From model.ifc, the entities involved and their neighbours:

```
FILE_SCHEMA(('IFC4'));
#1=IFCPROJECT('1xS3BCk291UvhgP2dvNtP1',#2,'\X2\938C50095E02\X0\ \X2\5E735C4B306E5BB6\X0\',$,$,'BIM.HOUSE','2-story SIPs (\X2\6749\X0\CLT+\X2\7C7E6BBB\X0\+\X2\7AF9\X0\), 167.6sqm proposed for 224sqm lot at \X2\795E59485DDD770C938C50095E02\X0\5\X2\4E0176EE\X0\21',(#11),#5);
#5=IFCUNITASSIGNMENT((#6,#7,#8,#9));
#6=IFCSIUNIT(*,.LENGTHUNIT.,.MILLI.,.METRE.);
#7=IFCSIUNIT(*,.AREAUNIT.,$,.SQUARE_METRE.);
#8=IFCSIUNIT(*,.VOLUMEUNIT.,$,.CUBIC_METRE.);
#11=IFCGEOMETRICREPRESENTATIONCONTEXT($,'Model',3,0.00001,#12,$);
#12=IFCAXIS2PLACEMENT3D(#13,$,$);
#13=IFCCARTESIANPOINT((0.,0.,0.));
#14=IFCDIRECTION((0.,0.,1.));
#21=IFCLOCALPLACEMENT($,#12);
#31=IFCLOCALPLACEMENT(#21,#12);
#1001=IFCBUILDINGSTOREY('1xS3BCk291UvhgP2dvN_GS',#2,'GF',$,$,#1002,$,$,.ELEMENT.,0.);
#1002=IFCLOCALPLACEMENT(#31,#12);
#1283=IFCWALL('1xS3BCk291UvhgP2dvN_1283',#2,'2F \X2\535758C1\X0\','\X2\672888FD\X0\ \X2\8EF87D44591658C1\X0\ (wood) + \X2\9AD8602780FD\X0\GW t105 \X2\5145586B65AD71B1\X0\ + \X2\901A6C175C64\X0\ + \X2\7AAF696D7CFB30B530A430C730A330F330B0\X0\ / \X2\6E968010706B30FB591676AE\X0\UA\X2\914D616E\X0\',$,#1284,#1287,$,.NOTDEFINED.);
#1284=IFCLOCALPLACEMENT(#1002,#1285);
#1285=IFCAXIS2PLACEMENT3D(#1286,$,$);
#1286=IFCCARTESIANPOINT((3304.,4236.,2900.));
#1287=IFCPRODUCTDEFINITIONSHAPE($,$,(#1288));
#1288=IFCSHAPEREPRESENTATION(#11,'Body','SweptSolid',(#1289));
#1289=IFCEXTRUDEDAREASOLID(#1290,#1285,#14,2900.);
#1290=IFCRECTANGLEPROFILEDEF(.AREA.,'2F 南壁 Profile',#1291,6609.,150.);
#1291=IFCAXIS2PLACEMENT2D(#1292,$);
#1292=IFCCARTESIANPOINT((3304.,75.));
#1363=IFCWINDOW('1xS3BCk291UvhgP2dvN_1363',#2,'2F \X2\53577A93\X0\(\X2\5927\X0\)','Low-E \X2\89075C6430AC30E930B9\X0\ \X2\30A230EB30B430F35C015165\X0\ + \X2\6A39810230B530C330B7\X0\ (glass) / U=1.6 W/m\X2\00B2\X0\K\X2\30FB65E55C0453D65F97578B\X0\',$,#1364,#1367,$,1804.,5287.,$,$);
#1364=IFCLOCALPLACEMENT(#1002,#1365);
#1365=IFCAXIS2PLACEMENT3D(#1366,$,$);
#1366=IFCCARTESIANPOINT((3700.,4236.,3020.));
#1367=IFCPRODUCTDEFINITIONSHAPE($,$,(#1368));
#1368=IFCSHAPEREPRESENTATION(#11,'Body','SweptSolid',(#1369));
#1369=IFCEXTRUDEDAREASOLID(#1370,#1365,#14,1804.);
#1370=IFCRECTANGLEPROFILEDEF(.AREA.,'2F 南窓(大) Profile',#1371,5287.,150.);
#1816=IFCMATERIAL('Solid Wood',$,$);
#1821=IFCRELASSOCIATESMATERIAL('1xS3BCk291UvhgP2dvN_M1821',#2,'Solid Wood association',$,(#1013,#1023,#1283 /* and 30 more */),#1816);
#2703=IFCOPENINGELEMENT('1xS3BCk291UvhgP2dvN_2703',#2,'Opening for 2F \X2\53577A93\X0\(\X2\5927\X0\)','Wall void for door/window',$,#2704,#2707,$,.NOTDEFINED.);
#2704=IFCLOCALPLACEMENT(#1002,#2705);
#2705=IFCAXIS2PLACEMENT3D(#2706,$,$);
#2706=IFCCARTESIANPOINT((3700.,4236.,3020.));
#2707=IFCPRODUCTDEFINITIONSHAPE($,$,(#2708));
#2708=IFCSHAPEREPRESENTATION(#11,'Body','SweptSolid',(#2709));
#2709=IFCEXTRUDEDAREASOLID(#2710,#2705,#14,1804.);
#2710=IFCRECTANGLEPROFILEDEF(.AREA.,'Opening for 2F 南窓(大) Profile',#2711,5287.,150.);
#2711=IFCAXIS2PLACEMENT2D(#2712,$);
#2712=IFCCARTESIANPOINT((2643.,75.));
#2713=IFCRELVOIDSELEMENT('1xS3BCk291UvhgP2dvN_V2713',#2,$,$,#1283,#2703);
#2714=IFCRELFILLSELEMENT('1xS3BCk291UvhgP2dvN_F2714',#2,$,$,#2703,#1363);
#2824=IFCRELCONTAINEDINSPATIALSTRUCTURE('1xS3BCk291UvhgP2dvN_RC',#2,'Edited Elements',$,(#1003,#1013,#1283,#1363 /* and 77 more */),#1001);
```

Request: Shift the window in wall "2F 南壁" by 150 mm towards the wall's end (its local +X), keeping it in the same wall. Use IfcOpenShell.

```python
import ifcopenshell
import ifcopenshell.api.geometry
import ifcopenshell.util.placement
import ifcopenshell.util.unit

model = ifcopenshell.open("model.ifc")
unit_scale = ifcopenshell.util.unit.calculate_unit_scale(model)

window = model.by_guid("1xS3BCk291UvhgP2dvN_1363")
opening = window.FillsVoids[0].RelatingOpeningElement
wall = opening.VoidsElements[0].RelatingBuildingElement

wall_matrix = ifcopenshell.util.placement.get_local_placement(wall.ObjectPlacement)
shift = wall_matrix[:3, 0] * 0.15 / unit_scale
before = ifcopenshell.util.placement.get_local_placement(window.ObjectPlacement)[:3, 3].copy()

# The window is not placed relative to its opening, so move both.
for product in (opening, window):
    matrix = ifcopenshell.util.placement.get_local_placement(product.ObjectPlacement)
    matrix[:3, 3] += shift
    ifcopenshell.api.geometry.edit_object_placement(model, product=product, matrix=matrix, is_si=False)

after = ifcopenshell.util.placement.get_local_placement(window.ObjectPlacement)[:3, 3]
print("window moved by", (after - before).round(3) + 0.0)

model.write("model_updated.ifc")
```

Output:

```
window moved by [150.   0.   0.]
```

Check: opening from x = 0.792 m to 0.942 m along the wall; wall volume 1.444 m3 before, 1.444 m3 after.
